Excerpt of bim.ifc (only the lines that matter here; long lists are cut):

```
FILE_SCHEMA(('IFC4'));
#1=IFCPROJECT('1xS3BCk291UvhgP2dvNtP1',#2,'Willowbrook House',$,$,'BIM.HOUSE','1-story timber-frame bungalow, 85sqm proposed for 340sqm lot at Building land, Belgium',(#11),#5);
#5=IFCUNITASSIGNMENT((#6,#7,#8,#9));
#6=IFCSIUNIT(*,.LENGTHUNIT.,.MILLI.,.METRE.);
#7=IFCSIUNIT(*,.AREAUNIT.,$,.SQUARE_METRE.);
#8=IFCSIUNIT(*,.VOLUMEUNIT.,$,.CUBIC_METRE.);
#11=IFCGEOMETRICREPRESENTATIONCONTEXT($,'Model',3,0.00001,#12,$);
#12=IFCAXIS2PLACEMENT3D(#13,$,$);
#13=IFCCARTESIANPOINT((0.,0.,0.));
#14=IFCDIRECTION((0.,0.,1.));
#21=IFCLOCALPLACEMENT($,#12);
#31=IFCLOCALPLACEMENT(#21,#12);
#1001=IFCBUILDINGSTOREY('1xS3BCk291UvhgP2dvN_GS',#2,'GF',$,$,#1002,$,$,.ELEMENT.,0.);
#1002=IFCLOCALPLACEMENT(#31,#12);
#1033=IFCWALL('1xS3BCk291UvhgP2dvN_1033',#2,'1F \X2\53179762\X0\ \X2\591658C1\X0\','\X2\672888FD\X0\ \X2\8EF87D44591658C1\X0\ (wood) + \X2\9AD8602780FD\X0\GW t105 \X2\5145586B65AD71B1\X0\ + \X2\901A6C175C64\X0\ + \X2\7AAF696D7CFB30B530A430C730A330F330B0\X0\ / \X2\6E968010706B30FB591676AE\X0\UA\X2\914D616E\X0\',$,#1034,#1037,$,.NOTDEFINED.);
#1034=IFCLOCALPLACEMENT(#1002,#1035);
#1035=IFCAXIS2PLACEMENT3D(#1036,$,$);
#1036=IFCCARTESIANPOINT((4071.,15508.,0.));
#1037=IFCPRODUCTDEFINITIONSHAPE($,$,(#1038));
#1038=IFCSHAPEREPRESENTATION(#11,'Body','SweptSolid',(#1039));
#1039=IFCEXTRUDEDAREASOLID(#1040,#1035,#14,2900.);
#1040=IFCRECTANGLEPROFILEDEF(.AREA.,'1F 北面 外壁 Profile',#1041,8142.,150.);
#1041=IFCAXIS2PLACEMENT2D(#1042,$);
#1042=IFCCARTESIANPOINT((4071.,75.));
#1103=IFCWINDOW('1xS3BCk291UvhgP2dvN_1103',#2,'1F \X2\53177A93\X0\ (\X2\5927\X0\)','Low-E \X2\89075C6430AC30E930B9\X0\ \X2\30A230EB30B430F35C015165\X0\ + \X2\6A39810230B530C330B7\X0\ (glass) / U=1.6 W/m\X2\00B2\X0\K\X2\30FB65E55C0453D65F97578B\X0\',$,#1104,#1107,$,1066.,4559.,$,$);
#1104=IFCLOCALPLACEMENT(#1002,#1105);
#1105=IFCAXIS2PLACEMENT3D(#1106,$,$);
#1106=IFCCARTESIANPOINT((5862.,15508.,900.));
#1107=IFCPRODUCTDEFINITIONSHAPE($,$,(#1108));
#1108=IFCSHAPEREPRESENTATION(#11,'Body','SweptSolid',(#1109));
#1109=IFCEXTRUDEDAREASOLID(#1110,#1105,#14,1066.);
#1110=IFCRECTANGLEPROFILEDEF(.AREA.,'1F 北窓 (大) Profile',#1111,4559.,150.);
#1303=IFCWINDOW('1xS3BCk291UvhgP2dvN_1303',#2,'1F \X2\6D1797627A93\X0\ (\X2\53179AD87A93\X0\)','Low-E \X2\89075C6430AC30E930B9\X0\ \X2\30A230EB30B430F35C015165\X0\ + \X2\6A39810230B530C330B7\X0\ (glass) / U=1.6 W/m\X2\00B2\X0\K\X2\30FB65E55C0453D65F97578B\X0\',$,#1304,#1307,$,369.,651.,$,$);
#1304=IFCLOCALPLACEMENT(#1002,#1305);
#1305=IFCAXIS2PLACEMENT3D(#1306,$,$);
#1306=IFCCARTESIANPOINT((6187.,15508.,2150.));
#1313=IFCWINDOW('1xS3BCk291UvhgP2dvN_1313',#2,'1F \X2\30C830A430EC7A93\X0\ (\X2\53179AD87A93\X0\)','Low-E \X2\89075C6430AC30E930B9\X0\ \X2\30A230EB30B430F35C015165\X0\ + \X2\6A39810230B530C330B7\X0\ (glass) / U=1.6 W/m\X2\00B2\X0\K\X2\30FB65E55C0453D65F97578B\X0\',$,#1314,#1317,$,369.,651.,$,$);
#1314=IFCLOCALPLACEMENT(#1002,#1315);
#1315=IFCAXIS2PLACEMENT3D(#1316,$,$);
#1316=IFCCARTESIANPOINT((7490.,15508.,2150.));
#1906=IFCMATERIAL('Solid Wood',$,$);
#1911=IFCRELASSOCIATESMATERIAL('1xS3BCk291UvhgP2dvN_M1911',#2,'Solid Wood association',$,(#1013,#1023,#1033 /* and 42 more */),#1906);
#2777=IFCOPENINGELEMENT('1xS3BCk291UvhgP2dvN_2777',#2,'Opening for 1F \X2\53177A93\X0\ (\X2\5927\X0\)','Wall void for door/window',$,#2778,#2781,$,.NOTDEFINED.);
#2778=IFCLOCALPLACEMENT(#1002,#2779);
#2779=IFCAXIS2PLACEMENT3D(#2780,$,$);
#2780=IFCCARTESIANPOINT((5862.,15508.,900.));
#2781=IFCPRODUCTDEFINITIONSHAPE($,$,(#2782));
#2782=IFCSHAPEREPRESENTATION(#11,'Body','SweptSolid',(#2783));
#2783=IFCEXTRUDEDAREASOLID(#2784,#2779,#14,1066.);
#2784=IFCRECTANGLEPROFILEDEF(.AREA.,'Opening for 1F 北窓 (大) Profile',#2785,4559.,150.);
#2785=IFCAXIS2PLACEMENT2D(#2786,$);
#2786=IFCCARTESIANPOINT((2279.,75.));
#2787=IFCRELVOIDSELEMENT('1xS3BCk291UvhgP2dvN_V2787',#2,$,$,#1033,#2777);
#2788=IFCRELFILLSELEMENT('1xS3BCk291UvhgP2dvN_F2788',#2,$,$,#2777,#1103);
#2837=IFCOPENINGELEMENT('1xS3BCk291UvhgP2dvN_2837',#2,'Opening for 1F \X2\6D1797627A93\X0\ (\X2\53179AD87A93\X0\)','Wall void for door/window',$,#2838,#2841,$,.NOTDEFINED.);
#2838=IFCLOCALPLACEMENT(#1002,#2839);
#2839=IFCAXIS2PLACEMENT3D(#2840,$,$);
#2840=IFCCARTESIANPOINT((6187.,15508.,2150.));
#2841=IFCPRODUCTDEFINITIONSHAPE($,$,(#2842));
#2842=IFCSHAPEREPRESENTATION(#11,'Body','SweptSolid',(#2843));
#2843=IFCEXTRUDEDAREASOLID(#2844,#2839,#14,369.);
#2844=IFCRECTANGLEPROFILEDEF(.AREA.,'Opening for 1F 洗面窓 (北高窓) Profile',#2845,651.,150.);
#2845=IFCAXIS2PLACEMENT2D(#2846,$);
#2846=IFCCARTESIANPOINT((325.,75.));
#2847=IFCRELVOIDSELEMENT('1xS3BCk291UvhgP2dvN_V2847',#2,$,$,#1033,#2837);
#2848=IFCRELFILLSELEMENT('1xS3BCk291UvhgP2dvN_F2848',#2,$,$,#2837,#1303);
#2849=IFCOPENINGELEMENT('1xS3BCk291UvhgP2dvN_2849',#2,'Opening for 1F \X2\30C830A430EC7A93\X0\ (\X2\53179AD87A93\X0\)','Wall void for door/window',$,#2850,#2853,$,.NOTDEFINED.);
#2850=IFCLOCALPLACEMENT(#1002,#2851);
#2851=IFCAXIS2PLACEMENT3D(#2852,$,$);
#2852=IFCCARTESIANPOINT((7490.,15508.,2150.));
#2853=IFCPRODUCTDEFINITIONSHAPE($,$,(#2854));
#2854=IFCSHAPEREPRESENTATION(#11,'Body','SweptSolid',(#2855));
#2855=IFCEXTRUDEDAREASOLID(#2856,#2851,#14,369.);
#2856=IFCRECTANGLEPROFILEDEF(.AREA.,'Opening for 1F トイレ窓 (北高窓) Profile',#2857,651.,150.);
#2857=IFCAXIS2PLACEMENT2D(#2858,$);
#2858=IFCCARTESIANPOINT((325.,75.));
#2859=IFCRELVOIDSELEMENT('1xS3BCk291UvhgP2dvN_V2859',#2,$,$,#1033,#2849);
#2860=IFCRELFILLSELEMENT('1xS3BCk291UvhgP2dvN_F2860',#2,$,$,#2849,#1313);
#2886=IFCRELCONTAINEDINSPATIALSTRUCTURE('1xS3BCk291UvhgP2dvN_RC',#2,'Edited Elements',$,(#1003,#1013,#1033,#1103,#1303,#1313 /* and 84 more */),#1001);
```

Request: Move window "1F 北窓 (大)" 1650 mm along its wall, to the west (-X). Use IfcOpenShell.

```python
import ifcopenshell
import ifcopenshell.api.geometry
import ifcopenshell.util.placement
import ifcopenshell.util.unit

model = ifcopenshell.open("bim.ifc")
unit_scale = ifcopenshell.util.unit.calculate_unit_scale(model)

window = model.by_guid("1xS3BCk291UvhgP2dvN_1103")
opening = window.FillsVoids[0].RelatingOpeningElement
wall = opening.VoidsElements[0].RelatingBuildingElement

wall_matrix = ifcopenshell.util.placement.get_local_placement(wall.ObjectPlacement)
shift = wall_matrix[:3, 0] * -1.65 / unit_scale
before = ifcopenshell.util.placement.get_local_placement(window.ObjectPlacement)[:3, 3].copy()

# The window is not placed relative to its opening, so move both.
for product in (opening, window):
    matrix = ifcopenshell.util.placement.get_local_placement(product.ObjectPlacement)
    matrix[:3, 3] += shift
    ifcopenshell.api.geometry.edit_object_placement(model, product=product, matrix=matrix, is_si=False)

after = ifcopenshell.util.placement.get_local_placement(window.ObjectPlacement)[:3, 3]
print("window moved by", (after - before).round(3) + 0.0)

model.write("bim_rev.ifc")
```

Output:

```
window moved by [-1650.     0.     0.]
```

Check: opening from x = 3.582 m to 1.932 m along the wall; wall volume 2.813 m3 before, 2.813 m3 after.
